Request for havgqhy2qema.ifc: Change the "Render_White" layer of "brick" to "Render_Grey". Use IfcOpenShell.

First a look at what the model holds.

```python
import ifcopenshell
import ifcopenshell.util.element

model = ifcopenshell.open("havgqhy2qema.ifc")
print(model.schema)
for layer_set in model.by_type("IfcMaterialLayerSet"):
    if layer_set.LayerSetName == "brick":
        for layer in layer_set.MaterialLayers:
            print(layer.id(), layer.Material and layer.Material.Name, layer.LayerThickness, sep=" | ")
        print(len(ifcopenshell.util.element.get_elements_by_material(model, layer_set)), "elements and types use it")
print(sorted(m.Name for m in model.by_type("IfcMaterial") if m.Name)[:60])
```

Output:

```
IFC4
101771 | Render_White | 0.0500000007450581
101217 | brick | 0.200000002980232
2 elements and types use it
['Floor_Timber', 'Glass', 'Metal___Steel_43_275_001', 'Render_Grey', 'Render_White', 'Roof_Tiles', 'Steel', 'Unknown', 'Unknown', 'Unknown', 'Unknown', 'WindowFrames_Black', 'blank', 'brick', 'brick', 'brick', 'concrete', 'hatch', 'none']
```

```python
import ifcopenshell
import ifcopenshell.api.material

model = ifcopenshell.open("havgqhy2qema.ifc")

layer_set = next(s for s in model.by_type("IfcMaterialLayerSet") if s.LayerSetName == "brick")
layer = next(l for l in layer_set.MaterialLayers if l.Material and l.Material.Name == "Render_White")
material = next(m for m in model.by_type("IfcMaterial") if m.Name == "Render_Grey")

# Point this one layer at the other material; renaming the old one would change it everywhere.
ifcopenshell.api.material.edit_layer(model, layer=layer, attributes={}, material=material)

print([l.Material.Name if l.Material else None for l in layer_set.MaterialLayers])

model.write("havgqhy2qema-out.ifc")
```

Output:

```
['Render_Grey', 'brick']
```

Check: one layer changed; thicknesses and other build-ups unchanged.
